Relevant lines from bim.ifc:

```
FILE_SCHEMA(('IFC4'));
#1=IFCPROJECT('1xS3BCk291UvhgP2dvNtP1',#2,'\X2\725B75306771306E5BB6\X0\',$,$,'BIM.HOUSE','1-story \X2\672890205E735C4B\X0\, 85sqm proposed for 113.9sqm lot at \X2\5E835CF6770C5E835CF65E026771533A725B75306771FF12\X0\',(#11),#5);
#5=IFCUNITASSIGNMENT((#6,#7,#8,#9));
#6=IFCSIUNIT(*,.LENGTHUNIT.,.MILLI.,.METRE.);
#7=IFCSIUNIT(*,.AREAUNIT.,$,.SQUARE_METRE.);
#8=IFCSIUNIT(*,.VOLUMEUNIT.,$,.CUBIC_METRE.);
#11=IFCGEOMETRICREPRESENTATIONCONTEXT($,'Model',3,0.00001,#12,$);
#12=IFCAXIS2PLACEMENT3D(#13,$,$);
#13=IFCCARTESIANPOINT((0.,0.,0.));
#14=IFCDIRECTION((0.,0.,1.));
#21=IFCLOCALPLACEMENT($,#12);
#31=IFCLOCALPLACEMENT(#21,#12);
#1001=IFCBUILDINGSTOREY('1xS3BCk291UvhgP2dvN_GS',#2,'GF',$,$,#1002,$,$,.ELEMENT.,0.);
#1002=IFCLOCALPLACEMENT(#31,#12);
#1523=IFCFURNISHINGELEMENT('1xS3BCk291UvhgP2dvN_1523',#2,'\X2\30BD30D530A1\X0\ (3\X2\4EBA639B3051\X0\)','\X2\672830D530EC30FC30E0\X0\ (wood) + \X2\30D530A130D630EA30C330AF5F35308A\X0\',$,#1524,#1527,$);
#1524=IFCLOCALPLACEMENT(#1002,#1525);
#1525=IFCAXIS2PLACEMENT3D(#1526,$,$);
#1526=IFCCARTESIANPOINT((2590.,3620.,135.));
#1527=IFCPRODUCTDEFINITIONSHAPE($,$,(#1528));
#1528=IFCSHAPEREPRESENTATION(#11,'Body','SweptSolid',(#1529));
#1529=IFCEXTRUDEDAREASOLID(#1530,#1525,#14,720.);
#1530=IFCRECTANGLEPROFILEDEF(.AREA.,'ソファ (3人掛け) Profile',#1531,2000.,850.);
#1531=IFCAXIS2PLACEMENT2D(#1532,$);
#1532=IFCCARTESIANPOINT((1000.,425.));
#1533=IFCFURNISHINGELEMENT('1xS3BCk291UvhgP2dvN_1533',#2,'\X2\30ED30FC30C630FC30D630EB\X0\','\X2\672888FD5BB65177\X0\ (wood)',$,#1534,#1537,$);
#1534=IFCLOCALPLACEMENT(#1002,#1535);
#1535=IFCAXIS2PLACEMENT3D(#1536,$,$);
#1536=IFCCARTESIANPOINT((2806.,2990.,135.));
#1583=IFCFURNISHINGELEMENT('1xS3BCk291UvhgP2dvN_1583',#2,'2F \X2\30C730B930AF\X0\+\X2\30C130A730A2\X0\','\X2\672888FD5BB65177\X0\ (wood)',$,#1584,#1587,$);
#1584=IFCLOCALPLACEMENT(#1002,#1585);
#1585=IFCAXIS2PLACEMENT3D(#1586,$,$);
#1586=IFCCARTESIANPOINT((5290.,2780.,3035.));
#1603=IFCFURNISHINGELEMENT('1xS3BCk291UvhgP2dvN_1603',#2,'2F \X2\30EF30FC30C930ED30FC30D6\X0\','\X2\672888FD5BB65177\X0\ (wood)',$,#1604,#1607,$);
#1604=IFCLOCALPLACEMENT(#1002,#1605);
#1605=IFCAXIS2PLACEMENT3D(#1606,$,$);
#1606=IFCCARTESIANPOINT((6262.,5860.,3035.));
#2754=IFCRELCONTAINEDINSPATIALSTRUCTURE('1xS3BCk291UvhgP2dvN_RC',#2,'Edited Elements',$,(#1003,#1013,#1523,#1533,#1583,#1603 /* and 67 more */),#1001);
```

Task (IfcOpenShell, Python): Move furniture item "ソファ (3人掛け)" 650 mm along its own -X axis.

```python
import ifcopenshell
import ifcopenshell.api.geometry
import ifcopenshell.util.placement
import ifcopenshell.util.unit

model = ifcopenshell.open("bim.ifc")
unit_scale = ifcopenshell.util.unit.calculate_unit_scale(model)

item = model.by_guid("1xS3BCk291UvhgP2dvN_1523")
matrix = ifcopenshell.util.placement.get_local_placement(item.ObjectPlacement)
matrix[:3, 3] -= matrix[:3, 0] * 0.65 / unit_scale
ifcopenshell.api.geometry.edit_object_placement(model, product=item, matrix=matrix, is_si=False)

print(ifcopenshell.util.placement.get_local_placement(item.ObjectPlacement).round(3) + 0.0)

model.write("bim-out.ifc")
```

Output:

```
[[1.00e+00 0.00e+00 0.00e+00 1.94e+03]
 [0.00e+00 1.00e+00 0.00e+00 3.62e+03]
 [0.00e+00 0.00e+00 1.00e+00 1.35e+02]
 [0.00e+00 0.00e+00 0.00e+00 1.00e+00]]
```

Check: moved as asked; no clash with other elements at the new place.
